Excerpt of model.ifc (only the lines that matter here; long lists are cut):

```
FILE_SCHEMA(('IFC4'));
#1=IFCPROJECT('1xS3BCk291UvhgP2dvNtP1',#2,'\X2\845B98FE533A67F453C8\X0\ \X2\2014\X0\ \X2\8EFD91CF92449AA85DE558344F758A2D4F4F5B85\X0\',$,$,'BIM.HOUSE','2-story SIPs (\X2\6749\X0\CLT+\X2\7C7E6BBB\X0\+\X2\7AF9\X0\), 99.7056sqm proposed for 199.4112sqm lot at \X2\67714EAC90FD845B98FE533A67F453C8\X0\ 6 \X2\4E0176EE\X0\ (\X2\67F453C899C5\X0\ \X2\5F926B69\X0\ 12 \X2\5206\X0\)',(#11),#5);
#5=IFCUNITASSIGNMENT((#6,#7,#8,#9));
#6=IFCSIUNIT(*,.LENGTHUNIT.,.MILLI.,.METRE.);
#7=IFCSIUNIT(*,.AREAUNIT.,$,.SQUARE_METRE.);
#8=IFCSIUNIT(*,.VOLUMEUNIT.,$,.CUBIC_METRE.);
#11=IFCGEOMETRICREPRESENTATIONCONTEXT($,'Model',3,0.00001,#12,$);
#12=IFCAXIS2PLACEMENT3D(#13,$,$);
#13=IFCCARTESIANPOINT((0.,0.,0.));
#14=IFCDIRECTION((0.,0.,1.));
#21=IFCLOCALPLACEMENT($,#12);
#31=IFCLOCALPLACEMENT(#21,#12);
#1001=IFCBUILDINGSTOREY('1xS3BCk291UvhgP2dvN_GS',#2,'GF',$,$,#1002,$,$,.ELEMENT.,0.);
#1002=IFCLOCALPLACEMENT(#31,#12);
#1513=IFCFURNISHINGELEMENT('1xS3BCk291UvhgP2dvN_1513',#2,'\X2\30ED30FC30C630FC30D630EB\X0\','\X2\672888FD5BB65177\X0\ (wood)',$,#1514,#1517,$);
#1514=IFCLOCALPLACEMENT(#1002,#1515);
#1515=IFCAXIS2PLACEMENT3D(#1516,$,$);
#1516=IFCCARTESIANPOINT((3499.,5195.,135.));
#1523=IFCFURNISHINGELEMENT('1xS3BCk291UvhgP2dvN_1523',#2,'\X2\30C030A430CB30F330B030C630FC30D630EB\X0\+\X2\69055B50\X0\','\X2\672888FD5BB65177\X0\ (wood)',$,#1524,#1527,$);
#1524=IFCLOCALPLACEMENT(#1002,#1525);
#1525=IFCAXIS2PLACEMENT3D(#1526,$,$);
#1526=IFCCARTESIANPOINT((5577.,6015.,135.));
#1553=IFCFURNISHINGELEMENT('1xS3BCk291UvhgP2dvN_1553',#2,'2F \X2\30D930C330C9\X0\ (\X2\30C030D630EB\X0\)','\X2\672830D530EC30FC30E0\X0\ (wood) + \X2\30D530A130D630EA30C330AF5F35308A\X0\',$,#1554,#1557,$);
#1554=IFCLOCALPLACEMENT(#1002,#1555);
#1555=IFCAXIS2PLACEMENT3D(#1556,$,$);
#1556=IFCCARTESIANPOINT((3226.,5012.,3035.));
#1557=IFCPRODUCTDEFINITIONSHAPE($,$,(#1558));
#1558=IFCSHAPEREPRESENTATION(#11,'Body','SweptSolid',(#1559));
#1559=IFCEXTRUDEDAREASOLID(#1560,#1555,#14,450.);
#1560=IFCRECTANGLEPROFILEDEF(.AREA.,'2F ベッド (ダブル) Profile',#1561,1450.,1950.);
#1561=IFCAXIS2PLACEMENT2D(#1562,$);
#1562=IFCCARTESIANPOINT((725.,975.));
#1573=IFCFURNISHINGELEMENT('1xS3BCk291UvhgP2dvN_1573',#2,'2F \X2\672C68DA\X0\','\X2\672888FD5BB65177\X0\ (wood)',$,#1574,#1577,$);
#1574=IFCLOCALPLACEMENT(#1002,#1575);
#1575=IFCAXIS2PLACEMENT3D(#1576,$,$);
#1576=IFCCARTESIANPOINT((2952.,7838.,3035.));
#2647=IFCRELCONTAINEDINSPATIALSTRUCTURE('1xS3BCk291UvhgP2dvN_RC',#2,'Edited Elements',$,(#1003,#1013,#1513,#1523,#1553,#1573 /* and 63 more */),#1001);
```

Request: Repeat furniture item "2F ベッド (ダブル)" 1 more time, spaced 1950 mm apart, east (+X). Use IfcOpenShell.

```python
import numpy as np
import ifcopenshell
import ifcopenshell.api.geometry
import ifcopenshell.api.root
import ifcopenshell.util.element
import ifcopenshell.util.placement
import ifcopenshell.util.unit

model = ifcopenshell.open("model.ifc")
unit_scale = ifcopenshell.util.unit.calculate_unit_scale(model)


def reuse_history(source, copy):
    """copy_class also copies each property set's owner history, people and application; keep the originals."""
    for rel in copy.IsDefinedBy:
        if rel.is_a("IfcRelDefinesByProperties") and (history := rel.RelatingPropertyDefinition.OwnerHistory):
            rel.RelatingPropertyDefinition.OwnerHistory = source.OwnerHistory
            ifcopenshell.util.element.remove_deep2(model, history)


source = model.by_id(1553)
base = ifcopenshell.util.placement.get_local_placement(source.ObjectPlacement)
step = np.array([1.0, 0.0, 0.0]) * 1.95 / unit_scale

for i in range(1, 2):
    copy = ifcopenshell.api.root.copy_class(model, product=source)
    copy.Representation = ifcopenshell.util.element.copy_deep(
        model, source.Representation, exclude=["IfcGeometricRepresentationContext", "IfcRepresentationMap"]
    )
    reuse_history(source, copy)
    matrix = base.copy()
    matrix[:3, 3] += i * step
    print("added at", matrix[:3, 3].round(3) + 0.0)
    ifcopenshell.api.geometry.edit_object_placement(model, product=copy, matrix=matrix, is_si=False)

model.write("model_v2.ifc")
```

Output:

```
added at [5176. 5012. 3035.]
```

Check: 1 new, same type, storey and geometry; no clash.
